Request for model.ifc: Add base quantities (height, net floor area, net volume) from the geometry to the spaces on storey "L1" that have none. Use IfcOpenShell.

First a look at what the model holds.

```python
import ifcopenshell
import ifcopenshell.util.element
import ifcopenshell.util.unit

model = ifcopenshell.open("model.ifc")
print(model.schema)
for unit_type in ("LENGTHUNIT", "AREAUNIT", "VOLUMEUNIT"):
    print(unit_type, ifcopenshell.util.unit.calculate_unit_scale(model, unit_type))
storey = next(s for s in model.by_type("IfcBuildingStorey") if s.Name == "L1")
spaces = [e for e in ifcopenshell.util.element.get_decomposition(storey) if e.is_a("IfcSpace")]
for e in sorted(spaces, key=lambda e: e.id()):
    print(e.id(), e.is_a(), e.Name, list(ifcopenshell.util.element.get_psets(e, qtos_only=True)), sep=" | ")
```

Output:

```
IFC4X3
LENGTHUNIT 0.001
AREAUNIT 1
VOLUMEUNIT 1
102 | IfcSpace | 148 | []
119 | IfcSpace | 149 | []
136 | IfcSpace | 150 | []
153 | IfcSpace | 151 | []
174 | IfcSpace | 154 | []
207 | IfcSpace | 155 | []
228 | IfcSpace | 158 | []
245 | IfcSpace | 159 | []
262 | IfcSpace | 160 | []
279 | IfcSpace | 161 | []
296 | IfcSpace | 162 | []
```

```python
import ifcopenshell
import ifcopenshell.api.pset
import ifcopenshell.geom
import ifcopenshell.util.element
import ifcopenshell.util.shape
import ifcopenshell.util.unit

model = ifcopenshell.open("model.ifc")
unit_scale = ifcopenshell.util.unit.calculate_unit_scale(model)
area_scale = ifcopenshell.util.unit.calculate_unit_scale(model, "AREAUNIT")
volume_scale = ifcopenshell.util.unit.calculate_unit_scale(model, "VOLUMEUNIT")
settings = ifcopenshell.geom.settings()

storey = next(s for s in model.by_type("IfcBuildingStorey") if s.Name == "L1")
spaces = [e for e in ifcopenshell.util.element.get_decomposition(storey) if e.is_a("IfcSpace")]

for e in sorted(spaces, key=lambda e: e.id()):
    if ifcopenshell.util.element.get_psets(e, qtos_only=True, should_inherit=False):
        continue
    # Geometry comes back in metres, in the element's own axes.
    shape = ifcopenshell.geom.create_shape(settings, e)
    values = {
        "Height": ifcopenshell.util.shape.get_z(shape.geometry) / unit_scale,
        "NetFloorArea": ifcopenshell.util.shape.get_footprint_area(shape.geometry) / area_scale,
        "NetVolume": ifcopenshell.util.shape.get_volume(shape.geometry) / volume_scale,
    }
    qto = ifcopenshell.api.pset.add_qto(model, product=e, name="Qto_SpaceBaseQuantities")
    ifcopenshell.api.pset.edit_qto(model, qto=qto, properties=values)
    print(e.id(), {k: round(v, 3) for k, v in values.items()})

model.write("model_edited.ifc")
```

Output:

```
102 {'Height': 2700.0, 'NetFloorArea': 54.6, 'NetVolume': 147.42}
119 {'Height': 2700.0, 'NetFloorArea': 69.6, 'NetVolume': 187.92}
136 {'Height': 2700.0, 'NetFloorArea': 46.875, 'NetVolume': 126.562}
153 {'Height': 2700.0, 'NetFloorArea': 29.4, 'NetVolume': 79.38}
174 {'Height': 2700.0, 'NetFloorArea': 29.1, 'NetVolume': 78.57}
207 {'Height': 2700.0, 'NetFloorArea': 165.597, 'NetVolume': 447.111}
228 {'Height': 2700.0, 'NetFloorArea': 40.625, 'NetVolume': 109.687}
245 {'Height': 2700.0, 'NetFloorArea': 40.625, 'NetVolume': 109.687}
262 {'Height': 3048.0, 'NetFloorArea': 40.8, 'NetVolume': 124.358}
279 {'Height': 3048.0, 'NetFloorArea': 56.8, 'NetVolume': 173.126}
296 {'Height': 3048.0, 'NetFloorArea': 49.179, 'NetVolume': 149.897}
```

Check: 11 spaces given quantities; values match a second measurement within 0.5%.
